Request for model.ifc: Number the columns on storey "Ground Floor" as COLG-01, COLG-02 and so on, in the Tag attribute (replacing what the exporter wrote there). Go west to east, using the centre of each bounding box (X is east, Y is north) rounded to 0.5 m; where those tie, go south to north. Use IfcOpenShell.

First a look at what the model holds.

```python
import ifcopenshell
import ifcopenshell.util.element
import ifcopenshell.util.placement

model = ifcopenshell.open("model.ifc")
print(model.schema)
storey = next(s for s in model.by_type("IfcBuildingStorey") if s.Name == "Ground Floor")
columns = [e for e in ifcopenshell.util.element.get_decomposition(storey) if e.is_a("IfcColumn")]
for e in sorted(columns, key=lambda e: e.id()):
    origin = ifcopenshell.util.placement.get_local_placement(e.ObjectPlacement)[:3, 3]
    print(e.id(), e.Tag, e.Name, origin.round(2) + 0.0, sep=" | ")
```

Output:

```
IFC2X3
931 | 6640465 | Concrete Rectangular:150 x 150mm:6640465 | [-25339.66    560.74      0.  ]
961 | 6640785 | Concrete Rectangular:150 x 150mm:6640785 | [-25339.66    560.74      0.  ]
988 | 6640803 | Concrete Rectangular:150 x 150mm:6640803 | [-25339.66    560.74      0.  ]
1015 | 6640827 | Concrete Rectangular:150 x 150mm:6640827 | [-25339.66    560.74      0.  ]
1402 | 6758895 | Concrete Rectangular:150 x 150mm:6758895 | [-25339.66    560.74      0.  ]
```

```python
import ifcopenshell
import ifcopenshell.geom
import ifcopenshell.util.element
import ifcopenshell.util.shape

model = ifcopenshell.open("model.ifc")
settings = ifcopenshell.geom.settings()
settings.set("use-world-coords", True)


def centre(element):
    shape = ifcopenshell.geom.create_shape(settings, element)
    return ifcopenshell.util.shape.get_bbox_centroid(shape.geometry)


storey = next(s for s in model.by_type("IfcBuildingStorey") if s.Name == "Ground Floor")
columns = [e for e in ifcopenshell.util.element.get_decomposition(storey) if e.is_a("IfcColumn")]

# Insertion points can sit at a corner or the storey origin, so sort by the geometry (in metres).
centres = {e: centre(e) for e in columns}
columns.sort(key=lambda e: (round(centres[e][0] / 0.5), centres[e][1]))

for i, e in enumerate(columns, start=1):
    number = f"COLG-{i:02d}"
    e.Tag = number
    print(e.id(), number)

model.write("model_edited.ifc")
```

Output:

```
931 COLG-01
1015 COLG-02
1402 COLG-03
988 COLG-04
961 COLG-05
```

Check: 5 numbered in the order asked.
